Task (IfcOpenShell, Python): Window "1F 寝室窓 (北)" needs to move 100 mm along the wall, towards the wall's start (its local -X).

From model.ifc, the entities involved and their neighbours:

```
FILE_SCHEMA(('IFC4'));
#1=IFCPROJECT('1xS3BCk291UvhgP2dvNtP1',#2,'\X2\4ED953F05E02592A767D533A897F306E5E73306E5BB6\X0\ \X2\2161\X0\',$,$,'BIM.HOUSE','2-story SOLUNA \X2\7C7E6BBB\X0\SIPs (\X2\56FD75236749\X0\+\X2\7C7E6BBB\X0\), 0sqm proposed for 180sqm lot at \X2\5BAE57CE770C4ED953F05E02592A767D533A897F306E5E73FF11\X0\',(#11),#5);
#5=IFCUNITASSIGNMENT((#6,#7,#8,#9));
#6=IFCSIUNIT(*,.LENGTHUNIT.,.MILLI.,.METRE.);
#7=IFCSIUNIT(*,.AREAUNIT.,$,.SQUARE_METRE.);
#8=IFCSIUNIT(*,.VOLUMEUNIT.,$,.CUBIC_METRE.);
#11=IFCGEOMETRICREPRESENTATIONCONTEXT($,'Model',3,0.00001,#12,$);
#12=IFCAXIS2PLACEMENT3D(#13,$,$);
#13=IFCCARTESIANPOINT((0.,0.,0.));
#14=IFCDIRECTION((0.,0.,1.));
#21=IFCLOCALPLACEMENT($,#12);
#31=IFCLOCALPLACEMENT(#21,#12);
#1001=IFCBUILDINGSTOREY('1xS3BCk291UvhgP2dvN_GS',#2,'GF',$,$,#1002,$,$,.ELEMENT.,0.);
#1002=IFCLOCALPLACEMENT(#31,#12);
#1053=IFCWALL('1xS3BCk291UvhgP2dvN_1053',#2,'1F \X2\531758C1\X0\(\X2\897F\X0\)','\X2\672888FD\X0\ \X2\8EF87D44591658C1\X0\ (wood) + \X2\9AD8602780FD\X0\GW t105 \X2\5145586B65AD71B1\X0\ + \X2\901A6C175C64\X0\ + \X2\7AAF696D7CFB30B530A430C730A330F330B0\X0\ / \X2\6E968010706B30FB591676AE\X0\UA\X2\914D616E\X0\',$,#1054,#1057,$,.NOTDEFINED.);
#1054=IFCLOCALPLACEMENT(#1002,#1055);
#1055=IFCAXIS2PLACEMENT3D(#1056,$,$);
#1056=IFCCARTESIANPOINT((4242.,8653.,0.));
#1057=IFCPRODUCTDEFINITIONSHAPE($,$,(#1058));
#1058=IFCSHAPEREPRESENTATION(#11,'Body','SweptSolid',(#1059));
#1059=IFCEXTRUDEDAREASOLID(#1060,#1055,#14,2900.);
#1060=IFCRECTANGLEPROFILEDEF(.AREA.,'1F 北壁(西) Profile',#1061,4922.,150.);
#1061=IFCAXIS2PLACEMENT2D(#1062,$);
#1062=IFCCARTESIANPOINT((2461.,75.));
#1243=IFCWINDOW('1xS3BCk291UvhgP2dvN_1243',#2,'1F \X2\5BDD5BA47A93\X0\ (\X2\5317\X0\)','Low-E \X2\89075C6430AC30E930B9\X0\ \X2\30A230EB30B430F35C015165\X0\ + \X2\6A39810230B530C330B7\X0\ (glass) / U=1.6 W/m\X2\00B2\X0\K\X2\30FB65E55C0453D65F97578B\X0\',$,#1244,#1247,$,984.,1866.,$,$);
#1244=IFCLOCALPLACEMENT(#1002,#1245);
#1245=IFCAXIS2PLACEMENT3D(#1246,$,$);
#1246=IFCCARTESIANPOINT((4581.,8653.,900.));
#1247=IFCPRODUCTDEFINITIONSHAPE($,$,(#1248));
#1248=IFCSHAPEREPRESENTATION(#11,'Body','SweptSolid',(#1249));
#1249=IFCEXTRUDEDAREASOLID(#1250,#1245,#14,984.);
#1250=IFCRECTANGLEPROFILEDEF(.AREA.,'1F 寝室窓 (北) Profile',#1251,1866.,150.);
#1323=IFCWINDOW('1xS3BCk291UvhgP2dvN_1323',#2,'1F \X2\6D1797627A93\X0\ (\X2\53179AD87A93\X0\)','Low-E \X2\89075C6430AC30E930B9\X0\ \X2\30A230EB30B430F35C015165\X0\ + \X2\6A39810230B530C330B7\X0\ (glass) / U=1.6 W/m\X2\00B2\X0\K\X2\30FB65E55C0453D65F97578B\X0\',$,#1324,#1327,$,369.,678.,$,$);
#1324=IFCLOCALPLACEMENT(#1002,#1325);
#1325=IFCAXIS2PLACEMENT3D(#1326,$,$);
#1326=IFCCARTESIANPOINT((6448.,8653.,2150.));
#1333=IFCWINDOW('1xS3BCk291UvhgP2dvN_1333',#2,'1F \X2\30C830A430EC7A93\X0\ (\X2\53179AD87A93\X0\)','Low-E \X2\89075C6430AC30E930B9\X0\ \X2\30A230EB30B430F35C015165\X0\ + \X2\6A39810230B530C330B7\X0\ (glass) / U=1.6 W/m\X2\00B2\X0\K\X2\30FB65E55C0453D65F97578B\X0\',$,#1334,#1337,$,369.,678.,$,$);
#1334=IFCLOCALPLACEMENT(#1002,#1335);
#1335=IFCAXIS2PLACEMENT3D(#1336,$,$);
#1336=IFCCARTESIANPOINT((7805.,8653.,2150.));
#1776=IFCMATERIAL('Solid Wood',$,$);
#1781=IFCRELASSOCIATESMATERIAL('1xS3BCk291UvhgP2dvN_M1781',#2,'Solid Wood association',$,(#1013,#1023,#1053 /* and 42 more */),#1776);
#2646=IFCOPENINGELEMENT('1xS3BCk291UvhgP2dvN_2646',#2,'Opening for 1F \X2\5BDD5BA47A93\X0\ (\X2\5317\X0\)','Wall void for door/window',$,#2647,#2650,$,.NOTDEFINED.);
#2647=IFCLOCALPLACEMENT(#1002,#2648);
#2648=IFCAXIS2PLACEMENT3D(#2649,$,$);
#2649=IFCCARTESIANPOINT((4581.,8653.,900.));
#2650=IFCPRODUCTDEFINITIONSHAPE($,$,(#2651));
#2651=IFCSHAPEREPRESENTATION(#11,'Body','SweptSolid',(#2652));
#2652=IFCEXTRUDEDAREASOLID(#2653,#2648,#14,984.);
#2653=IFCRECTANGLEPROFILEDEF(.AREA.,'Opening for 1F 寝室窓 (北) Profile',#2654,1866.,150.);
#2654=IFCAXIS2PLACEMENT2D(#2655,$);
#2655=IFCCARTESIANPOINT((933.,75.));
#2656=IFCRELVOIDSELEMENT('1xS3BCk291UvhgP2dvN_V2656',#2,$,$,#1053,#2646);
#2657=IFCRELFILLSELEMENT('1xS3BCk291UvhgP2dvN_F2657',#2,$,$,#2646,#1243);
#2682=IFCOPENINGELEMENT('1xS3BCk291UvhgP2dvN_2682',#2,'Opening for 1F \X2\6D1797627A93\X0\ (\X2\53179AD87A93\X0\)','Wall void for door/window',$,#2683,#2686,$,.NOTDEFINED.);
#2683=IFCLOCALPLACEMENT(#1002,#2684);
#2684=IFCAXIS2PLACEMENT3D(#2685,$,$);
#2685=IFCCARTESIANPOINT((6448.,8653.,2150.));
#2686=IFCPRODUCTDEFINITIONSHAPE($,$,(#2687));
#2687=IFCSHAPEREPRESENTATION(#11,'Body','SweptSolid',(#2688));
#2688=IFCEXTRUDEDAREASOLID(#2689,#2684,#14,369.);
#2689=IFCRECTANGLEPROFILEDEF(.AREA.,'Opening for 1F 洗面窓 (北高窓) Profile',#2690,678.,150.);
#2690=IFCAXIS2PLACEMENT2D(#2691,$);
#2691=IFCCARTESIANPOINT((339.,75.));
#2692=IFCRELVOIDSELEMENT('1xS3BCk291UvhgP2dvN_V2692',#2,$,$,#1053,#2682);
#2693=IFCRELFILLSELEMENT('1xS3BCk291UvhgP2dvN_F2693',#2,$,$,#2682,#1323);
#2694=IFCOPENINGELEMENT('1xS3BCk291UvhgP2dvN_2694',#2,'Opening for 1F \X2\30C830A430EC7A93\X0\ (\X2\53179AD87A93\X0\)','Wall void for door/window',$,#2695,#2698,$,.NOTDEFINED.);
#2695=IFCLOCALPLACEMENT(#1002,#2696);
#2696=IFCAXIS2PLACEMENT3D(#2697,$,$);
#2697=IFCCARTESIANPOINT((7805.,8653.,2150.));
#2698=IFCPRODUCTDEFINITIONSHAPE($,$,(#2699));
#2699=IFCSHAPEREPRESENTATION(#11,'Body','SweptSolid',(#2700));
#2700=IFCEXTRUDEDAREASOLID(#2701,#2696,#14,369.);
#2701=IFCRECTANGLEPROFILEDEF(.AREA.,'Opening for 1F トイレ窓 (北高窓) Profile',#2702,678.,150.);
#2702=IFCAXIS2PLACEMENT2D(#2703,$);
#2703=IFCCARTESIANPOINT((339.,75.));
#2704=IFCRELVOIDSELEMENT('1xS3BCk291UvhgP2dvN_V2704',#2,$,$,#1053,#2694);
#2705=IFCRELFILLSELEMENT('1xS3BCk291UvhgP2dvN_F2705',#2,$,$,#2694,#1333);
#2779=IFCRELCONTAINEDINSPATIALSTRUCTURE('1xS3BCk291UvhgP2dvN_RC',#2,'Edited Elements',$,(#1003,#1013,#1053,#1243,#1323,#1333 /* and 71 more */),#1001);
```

```python
import ifcopenshell
import ifcopenshell.api.geometry
import ifcopenshell.util.placement

model = ifcopenshell.open("model.ifc")

window = model.by_guid("1xS3BCk291UvhgP2dvN_1243")
opening = window.FillsVoids[0].RelatingOpeningElement
wall = opening.VoidsElements[0].RelatingBuildingElement

wall_matrix = ifcopenshell.util.placement.get_local_placement(wall.ObjectPlacement)
shift = wall_matrix[:3, 0] * -100.0
before = ifcopenshell.util.placement.get_local_placement(window.ObjectPlacement)[:3, 3].copy()

# The window is not placed relative to its opening, so move both.
for product in (opening, window):
    matrix = ifcopenshell.util.placement.get_local_placement(product.ObjectPlacement)
    matrix[:3, 3] += shift
    ifcopenshell.api.geometry.edit_object_placement(model, product=product, matrix=matrix, is_si=False)

after = ifcopenshell.util.placement.get_local_placement(window.ObjectPlacement)[:3, 3]
print("window moved by", (after - before).round(3) + 0.0)

model.write("model_updated.ifc")
```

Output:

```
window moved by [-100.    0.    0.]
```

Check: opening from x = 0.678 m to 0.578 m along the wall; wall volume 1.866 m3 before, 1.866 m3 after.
